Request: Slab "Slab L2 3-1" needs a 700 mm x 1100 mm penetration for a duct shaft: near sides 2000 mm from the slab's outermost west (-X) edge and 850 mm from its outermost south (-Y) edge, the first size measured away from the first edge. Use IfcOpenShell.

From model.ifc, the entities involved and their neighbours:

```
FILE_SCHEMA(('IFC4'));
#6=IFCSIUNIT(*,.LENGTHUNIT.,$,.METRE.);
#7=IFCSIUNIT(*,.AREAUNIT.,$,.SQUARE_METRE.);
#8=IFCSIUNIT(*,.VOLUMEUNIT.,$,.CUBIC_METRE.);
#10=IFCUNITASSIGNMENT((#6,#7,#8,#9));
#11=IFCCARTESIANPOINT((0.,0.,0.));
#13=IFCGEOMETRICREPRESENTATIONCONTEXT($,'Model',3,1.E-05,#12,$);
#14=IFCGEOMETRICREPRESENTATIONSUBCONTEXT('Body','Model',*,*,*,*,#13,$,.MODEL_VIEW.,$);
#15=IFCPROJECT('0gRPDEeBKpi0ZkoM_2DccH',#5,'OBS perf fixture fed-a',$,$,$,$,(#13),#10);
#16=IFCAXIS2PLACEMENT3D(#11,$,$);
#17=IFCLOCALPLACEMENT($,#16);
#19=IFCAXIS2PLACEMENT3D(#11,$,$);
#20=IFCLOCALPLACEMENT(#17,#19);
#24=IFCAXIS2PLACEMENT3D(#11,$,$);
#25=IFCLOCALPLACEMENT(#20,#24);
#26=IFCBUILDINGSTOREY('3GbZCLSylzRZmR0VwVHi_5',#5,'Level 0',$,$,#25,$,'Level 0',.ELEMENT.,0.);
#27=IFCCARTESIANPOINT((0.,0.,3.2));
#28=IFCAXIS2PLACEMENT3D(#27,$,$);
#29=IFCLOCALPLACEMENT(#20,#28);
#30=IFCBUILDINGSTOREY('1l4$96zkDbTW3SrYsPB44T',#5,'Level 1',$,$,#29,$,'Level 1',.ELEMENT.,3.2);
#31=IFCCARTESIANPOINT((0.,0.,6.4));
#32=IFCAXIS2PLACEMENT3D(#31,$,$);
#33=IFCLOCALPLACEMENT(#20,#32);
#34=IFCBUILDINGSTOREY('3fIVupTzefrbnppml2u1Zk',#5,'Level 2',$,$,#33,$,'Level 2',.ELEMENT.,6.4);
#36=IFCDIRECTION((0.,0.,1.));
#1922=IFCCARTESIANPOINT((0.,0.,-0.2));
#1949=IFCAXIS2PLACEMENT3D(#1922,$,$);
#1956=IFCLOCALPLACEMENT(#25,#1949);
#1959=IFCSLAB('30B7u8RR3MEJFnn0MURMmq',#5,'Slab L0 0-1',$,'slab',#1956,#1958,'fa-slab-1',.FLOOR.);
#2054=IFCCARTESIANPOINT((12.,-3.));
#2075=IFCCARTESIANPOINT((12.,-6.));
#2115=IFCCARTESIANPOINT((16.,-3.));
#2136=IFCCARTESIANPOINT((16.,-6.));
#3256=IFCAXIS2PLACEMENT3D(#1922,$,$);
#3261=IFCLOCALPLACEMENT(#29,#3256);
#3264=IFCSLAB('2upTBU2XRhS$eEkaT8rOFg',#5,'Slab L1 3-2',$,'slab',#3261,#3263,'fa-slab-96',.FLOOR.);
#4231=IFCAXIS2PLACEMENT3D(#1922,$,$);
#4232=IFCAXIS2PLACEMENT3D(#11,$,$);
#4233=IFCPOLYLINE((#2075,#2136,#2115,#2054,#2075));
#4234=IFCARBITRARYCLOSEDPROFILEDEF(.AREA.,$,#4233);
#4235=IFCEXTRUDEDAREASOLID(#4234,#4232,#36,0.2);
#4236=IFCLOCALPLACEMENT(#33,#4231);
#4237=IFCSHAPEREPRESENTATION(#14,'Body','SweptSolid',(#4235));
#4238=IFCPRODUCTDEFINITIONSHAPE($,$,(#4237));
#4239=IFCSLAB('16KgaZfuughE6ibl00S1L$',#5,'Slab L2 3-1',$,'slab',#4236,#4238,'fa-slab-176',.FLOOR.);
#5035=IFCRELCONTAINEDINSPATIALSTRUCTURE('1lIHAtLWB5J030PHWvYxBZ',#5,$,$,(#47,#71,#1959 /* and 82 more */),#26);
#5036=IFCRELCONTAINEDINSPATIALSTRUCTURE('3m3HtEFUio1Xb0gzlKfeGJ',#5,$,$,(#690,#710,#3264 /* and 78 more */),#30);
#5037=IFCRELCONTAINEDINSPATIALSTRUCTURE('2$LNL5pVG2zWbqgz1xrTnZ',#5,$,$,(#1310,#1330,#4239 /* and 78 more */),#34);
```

```python
import numpy as np
import ifcopenshell
import ifcopenshell.api.feature
import ifcopenshell.api.geometry
import ifcopenshell.api.root
import ifcopenshell.geom
import ifcopenshell.util.placement
import ifcopenshell.util.representation
import ifcopenshell.util.shape
import ifcopenshell.util.unit

model = ifcopenshell.open("model.ifc")
unit_scale = ifcopenshell.util.unit.calculate_unit_scale(model)
settings = ifcopenshell.geom.settings()


def volume(element):
    """Net volume in cubic metres, openings subtracted."""
    shape = ifcopenshell.geom.create_shape(settings, element)
    return ifcopenshell.util.shape.get_volume(shape.geometry)


slab = model.by_guid("16KgaZfuughE6ibl00S1L$")
before = volume(slab)

# Extent in the slab's own axes, in metres. The edges named are its -X and -Y sides.
slab_shape = ifcopenshell.geom.create_shape(settings, slab)
vertices = ifcopenshell.util.shape.get_vertices(slab_shape.geometry)
x_min, y_min, bottom = vertices.min(axis=0)
top = vertices[:, 2].max()

opening = ifcopenshell.api.root.create_entity(model, ifc_class="IfcOpeningElement", name="Duct shaft opening", predefined_type="OPENING")
context = ifcopenshell.util.representation.get_context(model, "Model", "Body", "MODEL_VIEW")
width, depth = 0.7, 1.1
outline = [(0.0, 0.0), (width, 0.0), (width, depth), (0.0, depth), (0.0, 0.0)]
# Overshoot both faces by 50 mm so the cut is clean.
shape = ifcopenshell.api.geometry.add_slab_representation(
    model, context=context, depth=top - bottom + 0.1, polyline=outline
)
ifcopenshell.api.geometry.assign_representation(model, product=opening, representation=shape)

matrix = ifcopenshell.util.placement.get_local_placement(slab.ObjectPlacement)
matrix[:, 3] = matrix @ np.append(np.array([x_min + 2, y_min + 0.85, bottom - 0.05]) / unit_scale, 1.0)
ifcopenshell.api.geometry.edit_object_placement(model, product=opening, matrix=matrix, is_si=False)
ifcopenshell.api.feature.add_feature(model, feature=opening, element=slab)

after = volume(slab)

print(f"slab volume {before:.3f} -> {after:.3f} m3")

model.write("model_v2.ifc")
```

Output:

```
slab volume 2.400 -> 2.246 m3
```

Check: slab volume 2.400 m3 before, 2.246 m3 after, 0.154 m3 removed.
